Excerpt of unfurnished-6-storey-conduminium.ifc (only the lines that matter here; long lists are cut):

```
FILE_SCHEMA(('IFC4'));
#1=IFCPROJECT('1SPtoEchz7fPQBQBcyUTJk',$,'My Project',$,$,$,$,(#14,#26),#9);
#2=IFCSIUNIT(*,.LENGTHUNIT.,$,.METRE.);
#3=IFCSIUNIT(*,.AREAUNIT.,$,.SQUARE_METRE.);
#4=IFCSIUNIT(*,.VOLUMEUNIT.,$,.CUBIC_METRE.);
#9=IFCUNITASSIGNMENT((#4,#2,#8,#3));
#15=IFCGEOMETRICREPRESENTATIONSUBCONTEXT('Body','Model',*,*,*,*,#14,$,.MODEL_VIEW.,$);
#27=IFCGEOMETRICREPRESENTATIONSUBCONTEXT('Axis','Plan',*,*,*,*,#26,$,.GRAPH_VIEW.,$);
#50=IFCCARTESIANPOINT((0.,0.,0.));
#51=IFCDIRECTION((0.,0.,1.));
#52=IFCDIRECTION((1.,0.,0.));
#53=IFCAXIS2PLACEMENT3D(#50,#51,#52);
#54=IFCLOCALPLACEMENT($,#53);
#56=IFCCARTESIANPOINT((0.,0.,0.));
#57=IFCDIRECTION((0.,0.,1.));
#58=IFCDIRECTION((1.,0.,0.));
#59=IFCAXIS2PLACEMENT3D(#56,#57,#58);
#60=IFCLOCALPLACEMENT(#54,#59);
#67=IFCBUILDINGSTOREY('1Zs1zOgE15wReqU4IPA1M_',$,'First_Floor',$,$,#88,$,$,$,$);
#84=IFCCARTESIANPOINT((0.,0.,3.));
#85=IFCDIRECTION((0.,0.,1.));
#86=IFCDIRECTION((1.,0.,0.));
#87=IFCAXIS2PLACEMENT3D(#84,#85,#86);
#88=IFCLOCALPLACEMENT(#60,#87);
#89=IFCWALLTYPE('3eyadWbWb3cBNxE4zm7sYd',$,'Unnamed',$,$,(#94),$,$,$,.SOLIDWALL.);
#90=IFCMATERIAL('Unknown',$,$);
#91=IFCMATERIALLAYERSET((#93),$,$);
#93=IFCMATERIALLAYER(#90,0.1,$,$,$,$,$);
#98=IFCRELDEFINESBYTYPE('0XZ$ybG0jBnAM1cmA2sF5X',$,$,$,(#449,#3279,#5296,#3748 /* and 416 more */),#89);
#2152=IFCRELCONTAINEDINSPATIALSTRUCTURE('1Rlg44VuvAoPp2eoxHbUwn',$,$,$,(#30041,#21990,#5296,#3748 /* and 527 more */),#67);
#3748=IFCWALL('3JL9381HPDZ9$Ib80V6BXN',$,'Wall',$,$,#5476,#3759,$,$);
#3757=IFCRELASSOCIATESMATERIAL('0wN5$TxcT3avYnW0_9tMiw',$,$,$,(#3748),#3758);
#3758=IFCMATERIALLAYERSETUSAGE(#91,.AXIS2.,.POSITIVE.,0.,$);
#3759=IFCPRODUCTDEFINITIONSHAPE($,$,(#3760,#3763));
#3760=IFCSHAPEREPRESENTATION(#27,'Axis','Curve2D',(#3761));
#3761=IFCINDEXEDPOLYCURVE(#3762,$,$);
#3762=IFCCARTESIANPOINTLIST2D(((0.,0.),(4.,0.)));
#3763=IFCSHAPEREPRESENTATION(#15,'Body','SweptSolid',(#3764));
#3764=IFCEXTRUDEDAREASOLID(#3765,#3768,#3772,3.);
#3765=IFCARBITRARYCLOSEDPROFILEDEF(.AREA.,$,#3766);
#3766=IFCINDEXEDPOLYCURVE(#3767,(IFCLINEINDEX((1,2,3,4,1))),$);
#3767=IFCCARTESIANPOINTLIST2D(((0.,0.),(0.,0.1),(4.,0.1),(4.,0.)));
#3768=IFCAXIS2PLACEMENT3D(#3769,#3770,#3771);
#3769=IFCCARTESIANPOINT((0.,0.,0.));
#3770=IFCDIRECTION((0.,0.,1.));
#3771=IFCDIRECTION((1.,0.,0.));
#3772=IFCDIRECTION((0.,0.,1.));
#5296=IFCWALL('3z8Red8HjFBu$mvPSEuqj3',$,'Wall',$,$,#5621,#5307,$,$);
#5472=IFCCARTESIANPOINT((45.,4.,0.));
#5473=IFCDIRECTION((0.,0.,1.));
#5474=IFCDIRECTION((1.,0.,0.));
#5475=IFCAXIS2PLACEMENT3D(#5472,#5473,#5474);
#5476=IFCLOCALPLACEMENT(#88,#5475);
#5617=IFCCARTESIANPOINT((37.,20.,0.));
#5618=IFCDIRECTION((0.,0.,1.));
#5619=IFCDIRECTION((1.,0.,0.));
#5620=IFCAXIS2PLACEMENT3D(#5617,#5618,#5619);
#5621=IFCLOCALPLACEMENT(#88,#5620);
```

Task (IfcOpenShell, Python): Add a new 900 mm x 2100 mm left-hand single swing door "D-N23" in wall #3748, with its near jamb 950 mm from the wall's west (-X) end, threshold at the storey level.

```python
import numpy as np
import ifcopenshell
import ifcopenshell.api.feature
import ifcopenshell.api.geometry
import ifcopenshell.api.root
import ifcopenshell.api.spatial
import ifcopenshell.geom
import ifcopenshell.util.element
import ifcopenshell.util.placement
import ifcopenshell.util.representation
import ifcopenshell.util.shape
import ifcopenshell.util.unit

model = ifcopenshell.open("unfurnished-6-storey-conduminium.ifc")
unit_scale = ifcopenshell.util.unit.calculate_unit_scale(model)
settings = ifcopenshell.geom.settings()


def volume(element):
    """Net volume in cubic metres, openings subtracted."""
    shape = ifcopenshell.geom.create_shape(settings, element)
    return ifcopenshell.util.shape.get_volume(shape.geometry)


wall = model.by_id(3748)
storey = ifcopenshell.util.element.get_container(wall, ifc_class="IfcBuildingStorey")
context = ifcopenshell.util.representation.get_context(model, "Model", "Body", "MODEL_VIEW")
before = volume(wall)

width, height, from_end, sill = 0.9, 2.1, 0.95, 0.0  # metres

# The wall runs along its own X axis, and the end named is its -X end.
wall_shape = ifcopenshell.geom.create_shape(settings, wall)
x, y, z = ifcopenshell.util.shape.get_vertices(wall_shape.geometry).T
start = x.min() + from_end
face, thickness = float(y.min()), float(y.max() - y.min())
wall_matrix = ifcopenshell.util.placement.get_local_placement(wall.ObjectPlacement)
level = ifcopenshell.util.placement.get_local_placement(storey.ObjectPlacement)[2, 3]


def in_wall(x, y):
    """Placement at x, y metres in the wall's axes, at sill height."""
    matrix = wall_matrix.copy()
    matrix[:, 3] = wall_matrix @ np.array([x / unit_scale, y / unit_scale, 0.0, 1.0])
    matrix[2, 3] = level + sill / unit_scale
    return matrix


# Opening: a box that overshoots both wall faces by 50 mm.
opening = ifcopenshell.api.root.create_entity(model, ifc_class="IfcOpeningElement", predefined_type="OPENING")
box = ifcopenshell.api.geometry.add_wall_representation(
    model, context=context, length=width, height=height, thickness=thickness + 0.1
)
ifcopenshell.api.geometry.assign_representation(model, product=opening, representation=box)
ifcopenshell.api.geometry.edit_object_placement(model, product=opening, matrix=in_wall(start, face - 0.05), is_si=False)
ifcopenshell.api.feature.add_feature(model, feature=opening, element=wall)

door = ifcopenshell.api.root.create_entity(model, ifc_class="IfcDoor", name="D-N23", predefined_type="DOOR")
door.OverallWidth, door.OverallHeight = width / unit_scale, height / unit_scale
door.OperationType = "SINGLE_SWING_LEFT"
body = ifcopenshell.api.geometry.add_door_representation(
    model,
    context=context,
    overall_width=door.OverallWidth,
    overall_height=door.OverallHeight,
    operation_type="SINGLE_SWING_LEFT",
    lining_properties={"LiningDepth": thickness / unit_scale, "ThresholdDepth": thickness / unit_scale},
)
ifcopenshell.api.geometry.assign_representation(model, product=door, representation=body)
ifcopenshell.api.spatial.assign_container(model, products=[door], relating_structure=storey)
ifcopenshell.api.feature.add_filling(model, opening=opening, element=door)

# The lining spans the wall, so the door starts at the wall face.
ifcopenshell.api.geometry.edit_object_placement(model, product=door, matrix=in_wall(start, face), is_si=False)

after = volume(wall)

print(f"wall volume {before:.3f} -> {after:.3f} m3")

model.write("unfurnished-6-storey-conduminium_edited.ifc")
```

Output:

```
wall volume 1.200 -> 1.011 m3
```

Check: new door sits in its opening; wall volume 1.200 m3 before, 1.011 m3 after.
